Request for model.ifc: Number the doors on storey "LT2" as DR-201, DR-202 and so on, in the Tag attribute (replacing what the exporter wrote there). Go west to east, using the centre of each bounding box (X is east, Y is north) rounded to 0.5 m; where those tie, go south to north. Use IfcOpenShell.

First a look at what the model holds.

```python
import ifcopenshell
import ifcopenshell.util.element
import ifcopenshell.util.placement

model = ifcopenshell.open("model.ifc")
print(model.schema)
storey = next(s for s in model.by_type("IfcBuildingStorey") if s.Name == "LT2")
doors = [e for e in ifcopenshell.util.element.get_decomposition(storey) if e.is_a("IfcDoor")]
for e in sorted(doors, key=lambda e: e.id()):
    origin = ifcopenshell.util.placement.get_local_placement(e.ObjectPlacement)[:3, 3]
    print(e.id(), e.Tag, e.Name, origin.round(2) + 0.0, sep=" | ")
```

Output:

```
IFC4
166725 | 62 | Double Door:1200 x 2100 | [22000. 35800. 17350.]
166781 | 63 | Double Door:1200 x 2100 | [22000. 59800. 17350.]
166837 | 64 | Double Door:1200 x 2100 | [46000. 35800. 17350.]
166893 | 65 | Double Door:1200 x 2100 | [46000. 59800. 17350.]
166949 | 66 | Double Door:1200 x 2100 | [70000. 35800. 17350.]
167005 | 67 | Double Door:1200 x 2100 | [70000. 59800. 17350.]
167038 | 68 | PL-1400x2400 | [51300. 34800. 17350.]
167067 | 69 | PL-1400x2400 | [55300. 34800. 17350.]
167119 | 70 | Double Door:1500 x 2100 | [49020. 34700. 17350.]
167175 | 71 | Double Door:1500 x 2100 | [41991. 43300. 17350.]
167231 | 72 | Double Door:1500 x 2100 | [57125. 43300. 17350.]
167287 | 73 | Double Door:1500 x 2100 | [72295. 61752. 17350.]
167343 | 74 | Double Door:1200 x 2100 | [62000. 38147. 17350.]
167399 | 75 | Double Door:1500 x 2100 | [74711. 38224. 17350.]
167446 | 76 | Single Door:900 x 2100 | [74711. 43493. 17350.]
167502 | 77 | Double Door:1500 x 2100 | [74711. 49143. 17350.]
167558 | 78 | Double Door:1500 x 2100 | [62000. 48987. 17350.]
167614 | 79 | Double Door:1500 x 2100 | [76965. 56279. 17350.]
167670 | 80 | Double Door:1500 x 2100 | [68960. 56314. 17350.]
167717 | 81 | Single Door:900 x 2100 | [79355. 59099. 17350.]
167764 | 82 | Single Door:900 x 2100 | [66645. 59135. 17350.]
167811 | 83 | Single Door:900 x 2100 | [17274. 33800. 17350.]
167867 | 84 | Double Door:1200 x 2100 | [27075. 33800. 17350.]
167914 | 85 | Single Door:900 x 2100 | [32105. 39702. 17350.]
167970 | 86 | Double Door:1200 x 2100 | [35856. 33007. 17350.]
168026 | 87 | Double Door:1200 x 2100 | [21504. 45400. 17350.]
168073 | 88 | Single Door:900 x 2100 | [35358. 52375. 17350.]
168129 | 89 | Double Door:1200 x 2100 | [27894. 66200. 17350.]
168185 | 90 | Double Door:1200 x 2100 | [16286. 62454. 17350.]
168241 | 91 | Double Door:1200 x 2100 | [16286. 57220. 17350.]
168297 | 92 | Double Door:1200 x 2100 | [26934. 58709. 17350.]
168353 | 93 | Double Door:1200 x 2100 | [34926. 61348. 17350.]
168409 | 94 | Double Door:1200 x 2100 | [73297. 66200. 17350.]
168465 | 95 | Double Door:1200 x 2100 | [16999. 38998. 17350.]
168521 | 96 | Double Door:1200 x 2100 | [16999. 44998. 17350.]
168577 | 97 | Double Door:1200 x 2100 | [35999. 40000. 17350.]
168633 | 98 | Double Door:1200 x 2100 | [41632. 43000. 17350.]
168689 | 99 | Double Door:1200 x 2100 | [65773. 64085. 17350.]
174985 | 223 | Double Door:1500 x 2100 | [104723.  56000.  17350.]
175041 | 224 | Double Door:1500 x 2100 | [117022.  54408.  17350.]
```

```python
import ifcopenshell
import ifcopenshell.geom
import ifcopenshell.util.element
import ifcopenshell.util.shape

model = ifcopenshell.open("model.ifc")
settings = ifcopenshell.geom.settings()
settings.set("use-world-coords", True)


def centre(element):
    shape = ifcopenshell.geom.create_shape(settings, element)
    return ifcopenshell.util.shape.get_bbox_centroid(shape.geometry)


storey = next(s for s in model.by_type("IfcBuildingStorey") if s.Name == "LT2")
doors = [e for e in ifcopenshell.util.element.get_decomposition(storey) if e.is_a("IfcDoor")]

# Insertion points can sit at a corner or the storey origin, so sort by the geometry (in metres).
centres = {e: centre(e) for e in doors}
doors.sort(key=lambda e: (round(centres[e][0] / 0.5), centres[e][1]))

for i, e in enumerate(doors, start=1):
    number = f"DR-2{i:02d}"
    e.Tag = number
    print(e.id(), number)

model.write("model_rev.ifc")
```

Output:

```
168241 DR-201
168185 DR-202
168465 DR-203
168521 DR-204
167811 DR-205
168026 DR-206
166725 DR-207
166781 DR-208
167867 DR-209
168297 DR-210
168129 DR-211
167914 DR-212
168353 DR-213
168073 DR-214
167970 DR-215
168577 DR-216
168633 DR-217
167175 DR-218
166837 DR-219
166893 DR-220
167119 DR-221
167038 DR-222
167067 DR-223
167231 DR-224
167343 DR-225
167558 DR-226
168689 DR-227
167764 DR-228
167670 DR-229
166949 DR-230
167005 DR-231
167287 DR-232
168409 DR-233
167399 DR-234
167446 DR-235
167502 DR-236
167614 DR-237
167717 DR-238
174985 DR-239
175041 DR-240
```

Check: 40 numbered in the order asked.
